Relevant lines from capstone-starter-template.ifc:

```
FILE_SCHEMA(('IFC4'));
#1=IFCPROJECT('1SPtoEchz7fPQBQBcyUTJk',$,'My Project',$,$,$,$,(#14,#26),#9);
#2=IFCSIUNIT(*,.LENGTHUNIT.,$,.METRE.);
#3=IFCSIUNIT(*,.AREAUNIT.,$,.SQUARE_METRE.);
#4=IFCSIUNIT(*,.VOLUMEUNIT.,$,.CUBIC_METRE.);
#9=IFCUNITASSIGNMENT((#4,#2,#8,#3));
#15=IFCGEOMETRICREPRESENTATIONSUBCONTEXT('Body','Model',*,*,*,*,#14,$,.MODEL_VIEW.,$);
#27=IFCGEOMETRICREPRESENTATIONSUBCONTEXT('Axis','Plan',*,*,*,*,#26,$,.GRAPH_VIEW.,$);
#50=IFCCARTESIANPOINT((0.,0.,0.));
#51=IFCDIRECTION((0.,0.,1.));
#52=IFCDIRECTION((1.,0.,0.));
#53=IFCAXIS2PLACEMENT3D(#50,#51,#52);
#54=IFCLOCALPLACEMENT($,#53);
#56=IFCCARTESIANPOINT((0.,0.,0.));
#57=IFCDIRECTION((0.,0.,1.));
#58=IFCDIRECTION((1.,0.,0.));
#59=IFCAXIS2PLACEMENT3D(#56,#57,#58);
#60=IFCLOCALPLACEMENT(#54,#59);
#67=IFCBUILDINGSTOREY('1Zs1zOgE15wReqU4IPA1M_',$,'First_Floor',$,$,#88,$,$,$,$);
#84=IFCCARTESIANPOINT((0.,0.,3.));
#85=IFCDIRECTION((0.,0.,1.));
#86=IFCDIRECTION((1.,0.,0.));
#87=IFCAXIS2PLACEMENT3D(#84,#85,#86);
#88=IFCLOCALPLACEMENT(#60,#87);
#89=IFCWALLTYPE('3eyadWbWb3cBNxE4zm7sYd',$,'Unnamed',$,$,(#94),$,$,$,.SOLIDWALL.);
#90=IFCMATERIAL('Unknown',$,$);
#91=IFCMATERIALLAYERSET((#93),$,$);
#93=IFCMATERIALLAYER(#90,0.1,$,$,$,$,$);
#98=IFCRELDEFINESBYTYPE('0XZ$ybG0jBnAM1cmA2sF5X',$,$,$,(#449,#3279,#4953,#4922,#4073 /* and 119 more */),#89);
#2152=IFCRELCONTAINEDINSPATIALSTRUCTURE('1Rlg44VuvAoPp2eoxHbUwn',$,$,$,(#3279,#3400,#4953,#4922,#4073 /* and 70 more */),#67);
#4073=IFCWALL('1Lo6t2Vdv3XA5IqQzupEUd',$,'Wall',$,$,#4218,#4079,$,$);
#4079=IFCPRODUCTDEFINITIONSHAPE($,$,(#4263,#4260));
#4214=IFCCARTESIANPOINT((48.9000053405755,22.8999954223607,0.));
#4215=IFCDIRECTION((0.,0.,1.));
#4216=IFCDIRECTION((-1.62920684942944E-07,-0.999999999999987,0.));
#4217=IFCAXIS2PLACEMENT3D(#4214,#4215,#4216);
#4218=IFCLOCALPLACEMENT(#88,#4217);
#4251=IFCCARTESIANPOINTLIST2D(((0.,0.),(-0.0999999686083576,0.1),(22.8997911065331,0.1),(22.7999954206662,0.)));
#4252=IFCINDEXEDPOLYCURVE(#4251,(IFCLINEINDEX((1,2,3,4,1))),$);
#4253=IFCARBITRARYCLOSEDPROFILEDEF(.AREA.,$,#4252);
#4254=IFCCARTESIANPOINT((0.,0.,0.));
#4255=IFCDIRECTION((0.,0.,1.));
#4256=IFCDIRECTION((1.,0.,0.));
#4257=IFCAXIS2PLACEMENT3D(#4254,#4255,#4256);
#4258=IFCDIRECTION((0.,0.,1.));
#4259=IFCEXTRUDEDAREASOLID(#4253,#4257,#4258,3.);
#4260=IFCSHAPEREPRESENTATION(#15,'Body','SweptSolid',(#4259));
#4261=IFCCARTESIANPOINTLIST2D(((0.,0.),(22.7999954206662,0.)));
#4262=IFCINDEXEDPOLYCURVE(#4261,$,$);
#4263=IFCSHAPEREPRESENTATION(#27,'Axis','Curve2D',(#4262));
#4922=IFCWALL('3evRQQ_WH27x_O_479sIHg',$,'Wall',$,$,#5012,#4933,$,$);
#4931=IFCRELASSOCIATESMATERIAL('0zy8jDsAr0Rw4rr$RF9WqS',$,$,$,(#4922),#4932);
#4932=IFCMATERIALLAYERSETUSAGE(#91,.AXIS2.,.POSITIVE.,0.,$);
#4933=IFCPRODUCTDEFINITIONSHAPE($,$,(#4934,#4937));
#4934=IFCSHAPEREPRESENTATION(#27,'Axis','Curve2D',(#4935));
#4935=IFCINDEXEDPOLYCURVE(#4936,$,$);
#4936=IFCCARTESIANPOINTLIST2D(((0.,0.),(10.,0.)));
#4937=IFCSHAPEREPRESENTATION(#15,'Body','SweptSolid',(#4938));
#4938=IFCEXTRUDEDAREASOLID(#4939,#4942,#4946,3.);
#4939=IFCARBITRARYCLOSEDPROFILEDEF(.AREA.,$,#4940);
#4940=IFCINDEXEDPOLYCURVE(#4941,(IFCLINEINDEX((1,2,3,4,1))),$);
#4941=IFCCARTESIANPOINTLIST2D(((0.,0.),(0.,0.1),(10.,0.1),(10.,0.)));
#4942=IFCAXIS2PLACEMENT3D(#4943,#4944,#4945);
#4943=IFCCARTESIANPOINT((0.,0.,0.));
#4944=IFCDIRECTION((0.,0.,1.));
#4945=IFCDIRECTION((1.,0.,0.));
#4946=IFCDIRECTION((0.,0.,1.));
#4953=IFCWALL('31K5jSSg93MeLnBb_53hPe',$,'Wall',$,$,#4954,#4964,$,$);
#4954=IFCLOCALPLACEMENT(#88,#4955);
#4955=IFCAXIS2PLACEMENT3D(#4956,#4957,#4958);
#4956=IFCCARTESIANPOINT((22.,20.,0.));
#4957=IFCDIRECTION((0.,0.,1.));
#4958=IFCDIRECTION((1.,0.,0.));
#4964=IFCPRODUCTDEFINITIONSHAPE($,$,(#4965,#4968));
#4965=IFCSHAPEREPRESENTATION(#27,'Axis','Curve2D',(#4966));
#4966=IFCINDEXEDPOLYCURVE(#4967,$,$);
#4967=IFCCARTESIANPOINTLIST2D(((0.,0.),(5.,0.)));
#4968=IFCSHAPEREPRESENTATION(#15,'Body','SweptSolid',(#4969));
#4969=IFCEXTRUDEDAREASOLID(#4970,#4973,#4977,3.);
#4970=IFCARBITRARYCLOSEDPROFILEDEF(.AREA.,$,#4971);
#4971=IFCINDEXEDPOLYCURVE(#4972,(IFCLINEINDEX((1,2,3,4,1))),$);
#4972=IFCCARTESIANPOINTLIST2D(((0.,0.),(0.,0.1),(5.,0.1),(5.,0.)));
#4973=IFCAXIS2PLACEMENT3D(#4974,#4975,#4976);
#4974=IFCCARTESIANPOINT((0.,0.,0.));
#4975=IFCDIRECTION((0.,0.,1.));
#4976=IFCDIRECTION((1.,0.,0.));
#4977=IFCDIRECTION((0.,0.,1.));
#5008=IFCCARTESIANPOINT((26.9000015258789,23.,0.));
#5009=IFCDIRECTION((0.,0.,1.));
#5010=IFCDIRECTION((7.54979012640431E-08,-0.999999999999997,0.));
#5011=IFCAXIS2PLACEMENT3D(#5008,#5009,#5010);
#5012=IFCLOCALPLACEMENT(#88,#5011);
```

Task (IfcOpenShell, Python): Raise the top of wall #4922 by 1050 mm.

```python
import ifcopenshell
import ifcopenshell.geom
import ifcopenshell.util.representation
import ifcopenshell.util.shape

model = ifcopenshell.open("capstone-starter-template.ifc")
settings = ifcopenshell.geom.settings()


def volume(element):
    """Net volume in cubic metres, openings subtracted."""
    shape = ifcopenshell.geom.create_shape(settings, element)
    return ifcopenshell.util.shape.get_volume(shape.geometry)


wall = model.by_id(4922)
before = volume(wall)

body = ifcopenshell.util.representation.get_representation(wall, "Model", "Body")
solid = body.Items[0]
old_height = solid.Depth
solid.Depth += 1.05
after = volume(wall)

print(f"height {old_height:g} -> {solid.Depth:g}, volume {before:.3f} -> {after:.3f} m3")

model.write("capstone-starter-template-out.ifc")
```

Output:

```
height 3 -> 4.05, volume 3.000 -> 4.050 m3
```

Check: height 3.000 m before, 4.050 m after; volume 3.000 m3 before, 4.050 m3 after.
